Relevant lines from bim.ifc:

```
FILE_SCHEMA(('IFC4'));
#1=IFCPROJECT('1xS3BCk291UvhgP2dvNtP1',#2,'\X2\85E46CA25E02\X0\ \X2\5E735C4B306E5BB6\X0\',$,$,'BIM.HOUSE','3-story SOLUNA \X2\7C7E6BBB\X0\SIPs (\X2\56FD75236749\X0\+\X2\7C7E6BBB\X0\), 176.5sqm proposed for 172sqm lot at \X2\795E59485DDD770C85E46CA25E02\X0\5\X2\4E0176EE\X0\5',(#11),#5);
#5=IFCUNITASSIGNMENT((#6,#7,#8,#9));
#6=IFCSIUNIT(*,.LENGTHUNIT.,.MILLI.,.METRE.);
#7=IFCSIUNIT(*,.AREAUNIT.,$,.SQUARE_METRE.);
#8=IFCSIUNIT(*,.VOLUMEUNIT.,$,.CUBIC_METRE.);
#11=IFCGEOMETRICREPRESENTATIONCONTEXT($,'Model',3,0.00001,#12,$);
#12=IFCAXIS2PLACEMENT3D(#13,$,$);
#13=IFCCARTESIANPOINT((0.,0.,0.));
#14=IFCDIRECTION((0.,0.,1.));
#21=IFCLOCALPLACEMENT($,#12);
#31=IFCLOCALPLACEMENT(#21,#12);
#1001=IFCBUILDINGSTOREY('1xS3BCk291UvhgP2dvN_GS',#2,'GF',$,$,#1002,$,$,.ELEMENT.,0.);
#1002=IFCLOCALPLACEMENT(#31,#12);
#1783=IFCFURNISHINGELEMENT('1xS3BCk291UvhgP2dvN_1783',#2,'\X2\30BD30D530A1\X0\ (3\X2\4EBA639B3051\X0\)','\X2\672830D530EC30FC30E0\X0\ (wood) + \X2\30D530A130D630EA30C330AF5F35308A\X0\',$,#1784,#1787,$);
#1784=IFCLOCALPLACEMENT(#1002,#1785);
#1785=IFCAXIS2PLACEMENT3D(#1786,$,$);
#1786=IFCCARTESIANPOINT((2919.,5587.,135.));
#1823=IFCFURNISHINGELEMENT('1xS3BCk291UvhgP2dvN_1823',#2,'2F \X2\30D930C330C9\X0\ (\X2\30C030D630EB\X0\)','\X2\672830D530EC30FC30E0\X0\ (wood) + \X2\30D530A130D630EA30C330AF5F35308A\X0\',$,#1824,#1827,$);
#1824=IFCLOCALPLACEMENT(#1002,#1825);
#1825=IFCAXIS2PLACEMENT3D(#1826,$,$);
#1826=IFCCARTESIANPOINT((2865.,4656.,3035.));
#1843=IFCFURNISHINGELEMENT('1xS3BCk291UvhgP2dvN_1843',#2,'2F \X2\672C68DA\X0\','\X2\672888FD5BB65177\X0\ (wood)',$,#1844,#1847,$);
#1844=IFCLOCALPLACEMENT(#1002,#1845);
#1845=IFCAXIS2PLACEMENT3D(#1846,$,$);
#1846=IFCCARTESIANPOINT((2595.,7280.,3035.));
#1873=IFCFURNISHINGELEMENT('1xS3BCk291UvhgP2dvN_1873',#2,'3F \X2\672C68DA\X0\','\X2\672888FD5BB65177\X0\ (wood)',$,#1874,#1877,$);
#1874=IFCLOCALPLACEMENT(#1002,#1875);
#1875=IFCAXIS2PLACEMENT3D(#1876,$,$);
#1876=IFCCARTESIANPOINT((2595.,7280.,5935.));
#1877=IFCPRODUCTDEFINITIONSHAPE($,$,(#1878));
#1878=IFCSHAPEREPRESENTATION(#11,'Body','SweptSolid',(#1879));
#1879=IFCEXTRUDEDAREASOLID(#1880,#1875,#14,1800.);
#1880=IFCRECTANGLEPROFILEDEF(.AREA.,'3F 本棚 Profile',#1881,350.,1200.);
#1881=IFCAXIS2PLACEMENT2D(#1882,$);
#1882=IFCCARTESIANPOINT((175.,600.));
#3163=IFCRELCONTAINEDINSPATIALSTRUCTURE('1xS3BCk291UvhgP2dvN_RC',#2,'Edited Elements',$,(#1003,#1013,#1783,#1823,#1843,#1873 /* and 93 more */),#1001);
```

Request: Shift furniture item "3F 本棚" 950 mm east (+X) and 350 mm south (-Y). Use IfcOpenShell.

```python
import ifcopenshell
import ifcopenshell.api.geometry
import ifcopenshell.util.placement
import ifcopenshell.util.unit

model = ifcopenshell.open("bim.ifc")
unit_scale = ifcopenshell.util.unit.calculate_unit_scale(model)

item = model.by_guid("1xS3BCk291UvhgP2dvN_1873")
matrix = ifcopenshell.util.placement.get_local_placement(item.ObjectPlacement)
matrix[0, 3] += 0.95 / unit_scale
matrix[1, 3] -= 0.35 / unit_scale
ifcopenshell.api.geometry.edit_object_placement(model, product=item, matrix=matrix, is_si=False)

print(ifcopenshell.util.placement.get_local_placement(item.ObjectPlacement).round(3) + 0.0)

model.write("bim_rev.ifc")
```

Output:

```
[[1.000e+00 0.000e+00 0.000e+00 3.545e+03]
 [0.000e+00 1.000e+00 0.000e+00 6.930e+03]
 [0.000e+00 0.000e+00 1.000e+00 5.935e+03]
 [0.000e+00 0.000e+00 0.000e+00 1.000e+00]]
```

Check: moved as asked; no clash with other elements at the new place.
